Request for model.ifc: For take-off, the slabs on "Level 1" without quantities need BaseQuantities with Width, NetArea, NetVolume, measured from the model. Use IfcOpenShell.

First a look at what the model holds.

```python
import ifcopenshell
import ifcopenshell.util.element
import ifcopenshell.util.unit

model = ifcopenshell.open("model.ifc")
print(model.schema)
for unit_type in ("LENGTHUNIT", "AREAUNIT", "VOLUMEUNIT"):
    print(unit_type, ifcopenshell.util.unit.calculate_unit_scale(model, unit_type))
storey = next(s for s in model.by_type("IfcBuildingStorey") if s.Name == "Level 1")
slabs = [e for e in ifcopenshell.util.element.get_decomposition(storey) if e.is_a("IfcSlab")]
for e in sorted(slabs, key=lambda e: e.id()):
    print(e.id(), e.is_a(), e.Name, list(ifcopenshell.util.element.get_psets(e, qtos_only=True)), sep=" | ")
```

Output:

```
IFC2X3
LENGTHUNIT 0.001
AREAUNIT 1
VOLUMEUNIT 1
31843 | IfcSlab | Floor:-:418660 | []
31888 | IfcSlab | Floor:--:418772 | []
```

```python
import ifcopenshell
import ifcopenshell.api.pset
import ifcopenshell.geom
import ifcopenshell.util.element
import ifcopenshell.util.shape
import ifcopenshell.util.unit

model = ifcopenshell.open("model.ifc")
unit_scale = ifcopenshell.util.unit.calculate_unit_scale(model)
area_scale = ifcopenshell.util.unit.calculate_unit_scale(model, "AREAUNIT")
volume_scale = ifcopenshell.util.unit.calculate_unit_scale(model, "VOLUMEUNIT")
settings = ifcopenshell.geom.settings()

storey = next(s for s in model.by_type("IfcBuildingStorey") if s.Name == "Level 1")
slabs = [e for e in ifcopenshell.util.element.get_decomposition(storey) if e.is_a("IfcSlab")]

for e in sorted(slabs, key=lambda e: e.id()):
    if ifcopenshell.util.element.get_psets(e, qtos_only=True, should_inherit=False):
        continue
    # Geometry comes back in metres, in the element's own axes.
    shape = ifcopenshell.geom.create_shape(settings, e)
    values = {
        "Width": ifcopenshell.util.shape.get_z(shape.geometry) / unit_scale,
        "NetArea": ifcopenshell.util.shape.get_footprint_area(shape.geometry) / area_scale,
        "NetVolume": ifcopenshell.util.shape.get_volume(shape.geometry) / volume_scale,
    }
    qto = ifcopenshell.api.pset.add_qto(model, product=e, name="BaseQuantities")
    ifcopenshell.api.pset.edit_qto(model, qto=qto, properties=values)
    print(e.id(), {k: round(v, 3) for k, v in values.items()})

model.write("model_edited.ifc")
```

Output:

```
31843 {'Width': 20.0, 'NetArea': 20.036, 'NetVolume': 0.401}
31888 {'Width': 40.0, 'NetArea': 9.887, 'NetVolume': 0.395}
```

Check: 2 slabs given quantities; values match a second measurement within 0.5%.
